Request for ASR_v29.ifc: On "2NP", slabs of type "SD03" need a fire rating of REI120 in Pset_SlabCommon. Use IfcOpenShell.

First a look at what the model holds.

```python
import ifcopenshell
import ifcopenshell.util.element

model = ifcopenshell.open("ASR_v29.ifc")
print(model.schema)
storey = next(s for s in model.by_type("IfcBuildingStorey") if s.Name == "2NP")
slabs = [e for e in ifcopenshell.util.element.get_decomposition(storey) if e.is_a("IfcSlab")]
seen = {}
for e in slabs:
    element_type = ifcopenshell.util.element.get_type(e)
    key = (element_type.Name if element_type != e and element_type else None, ifcopenshell.util.element.get_pset(e, "Pset_SlabCommon", "FireRating"))
    seen[key] = seen.get(key, 0) + 1
for (name, value), count in sorted(seen.items(), key=str):
    print(count, "x", name, "|", value)
```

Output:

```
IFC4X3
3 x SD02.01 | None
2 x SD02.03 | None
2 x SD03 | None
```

```python
import ifcopenshell
import ifcopenshell.api.pset
import ifcopenshell.util.element

model = ifcopenshell.open("ASR_v29.ifc")

storey = next(s for s in model.by_type("IfcBuildingStorey") if s.Name == "2NP")
slabs = [e for e in ifcopenshell.util.element.get_decomposition(storey) if e.is_a("IfcSlab")]

count = 0
for e in slabs:
    element_type = ifcopenshell.util.element.get_type(e)
    if element_type in (None, e) or element_type.Name != "SD03":
        continue
    # add_pset returns the element's existing set when there is one.
    pset = ifcopenshell.api.pset.add_pset(model, product=e, name="Pset_SlabCommon")
    ifcopenshell.api.pset.edit_pset(model, pset=pset, properties={"FireRating": "REI120"})
    count += 1

print(count, "slabs updated")

model.write("ASR_v29-out.ifc")
```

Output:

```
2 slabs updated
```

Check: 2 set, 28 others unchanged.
